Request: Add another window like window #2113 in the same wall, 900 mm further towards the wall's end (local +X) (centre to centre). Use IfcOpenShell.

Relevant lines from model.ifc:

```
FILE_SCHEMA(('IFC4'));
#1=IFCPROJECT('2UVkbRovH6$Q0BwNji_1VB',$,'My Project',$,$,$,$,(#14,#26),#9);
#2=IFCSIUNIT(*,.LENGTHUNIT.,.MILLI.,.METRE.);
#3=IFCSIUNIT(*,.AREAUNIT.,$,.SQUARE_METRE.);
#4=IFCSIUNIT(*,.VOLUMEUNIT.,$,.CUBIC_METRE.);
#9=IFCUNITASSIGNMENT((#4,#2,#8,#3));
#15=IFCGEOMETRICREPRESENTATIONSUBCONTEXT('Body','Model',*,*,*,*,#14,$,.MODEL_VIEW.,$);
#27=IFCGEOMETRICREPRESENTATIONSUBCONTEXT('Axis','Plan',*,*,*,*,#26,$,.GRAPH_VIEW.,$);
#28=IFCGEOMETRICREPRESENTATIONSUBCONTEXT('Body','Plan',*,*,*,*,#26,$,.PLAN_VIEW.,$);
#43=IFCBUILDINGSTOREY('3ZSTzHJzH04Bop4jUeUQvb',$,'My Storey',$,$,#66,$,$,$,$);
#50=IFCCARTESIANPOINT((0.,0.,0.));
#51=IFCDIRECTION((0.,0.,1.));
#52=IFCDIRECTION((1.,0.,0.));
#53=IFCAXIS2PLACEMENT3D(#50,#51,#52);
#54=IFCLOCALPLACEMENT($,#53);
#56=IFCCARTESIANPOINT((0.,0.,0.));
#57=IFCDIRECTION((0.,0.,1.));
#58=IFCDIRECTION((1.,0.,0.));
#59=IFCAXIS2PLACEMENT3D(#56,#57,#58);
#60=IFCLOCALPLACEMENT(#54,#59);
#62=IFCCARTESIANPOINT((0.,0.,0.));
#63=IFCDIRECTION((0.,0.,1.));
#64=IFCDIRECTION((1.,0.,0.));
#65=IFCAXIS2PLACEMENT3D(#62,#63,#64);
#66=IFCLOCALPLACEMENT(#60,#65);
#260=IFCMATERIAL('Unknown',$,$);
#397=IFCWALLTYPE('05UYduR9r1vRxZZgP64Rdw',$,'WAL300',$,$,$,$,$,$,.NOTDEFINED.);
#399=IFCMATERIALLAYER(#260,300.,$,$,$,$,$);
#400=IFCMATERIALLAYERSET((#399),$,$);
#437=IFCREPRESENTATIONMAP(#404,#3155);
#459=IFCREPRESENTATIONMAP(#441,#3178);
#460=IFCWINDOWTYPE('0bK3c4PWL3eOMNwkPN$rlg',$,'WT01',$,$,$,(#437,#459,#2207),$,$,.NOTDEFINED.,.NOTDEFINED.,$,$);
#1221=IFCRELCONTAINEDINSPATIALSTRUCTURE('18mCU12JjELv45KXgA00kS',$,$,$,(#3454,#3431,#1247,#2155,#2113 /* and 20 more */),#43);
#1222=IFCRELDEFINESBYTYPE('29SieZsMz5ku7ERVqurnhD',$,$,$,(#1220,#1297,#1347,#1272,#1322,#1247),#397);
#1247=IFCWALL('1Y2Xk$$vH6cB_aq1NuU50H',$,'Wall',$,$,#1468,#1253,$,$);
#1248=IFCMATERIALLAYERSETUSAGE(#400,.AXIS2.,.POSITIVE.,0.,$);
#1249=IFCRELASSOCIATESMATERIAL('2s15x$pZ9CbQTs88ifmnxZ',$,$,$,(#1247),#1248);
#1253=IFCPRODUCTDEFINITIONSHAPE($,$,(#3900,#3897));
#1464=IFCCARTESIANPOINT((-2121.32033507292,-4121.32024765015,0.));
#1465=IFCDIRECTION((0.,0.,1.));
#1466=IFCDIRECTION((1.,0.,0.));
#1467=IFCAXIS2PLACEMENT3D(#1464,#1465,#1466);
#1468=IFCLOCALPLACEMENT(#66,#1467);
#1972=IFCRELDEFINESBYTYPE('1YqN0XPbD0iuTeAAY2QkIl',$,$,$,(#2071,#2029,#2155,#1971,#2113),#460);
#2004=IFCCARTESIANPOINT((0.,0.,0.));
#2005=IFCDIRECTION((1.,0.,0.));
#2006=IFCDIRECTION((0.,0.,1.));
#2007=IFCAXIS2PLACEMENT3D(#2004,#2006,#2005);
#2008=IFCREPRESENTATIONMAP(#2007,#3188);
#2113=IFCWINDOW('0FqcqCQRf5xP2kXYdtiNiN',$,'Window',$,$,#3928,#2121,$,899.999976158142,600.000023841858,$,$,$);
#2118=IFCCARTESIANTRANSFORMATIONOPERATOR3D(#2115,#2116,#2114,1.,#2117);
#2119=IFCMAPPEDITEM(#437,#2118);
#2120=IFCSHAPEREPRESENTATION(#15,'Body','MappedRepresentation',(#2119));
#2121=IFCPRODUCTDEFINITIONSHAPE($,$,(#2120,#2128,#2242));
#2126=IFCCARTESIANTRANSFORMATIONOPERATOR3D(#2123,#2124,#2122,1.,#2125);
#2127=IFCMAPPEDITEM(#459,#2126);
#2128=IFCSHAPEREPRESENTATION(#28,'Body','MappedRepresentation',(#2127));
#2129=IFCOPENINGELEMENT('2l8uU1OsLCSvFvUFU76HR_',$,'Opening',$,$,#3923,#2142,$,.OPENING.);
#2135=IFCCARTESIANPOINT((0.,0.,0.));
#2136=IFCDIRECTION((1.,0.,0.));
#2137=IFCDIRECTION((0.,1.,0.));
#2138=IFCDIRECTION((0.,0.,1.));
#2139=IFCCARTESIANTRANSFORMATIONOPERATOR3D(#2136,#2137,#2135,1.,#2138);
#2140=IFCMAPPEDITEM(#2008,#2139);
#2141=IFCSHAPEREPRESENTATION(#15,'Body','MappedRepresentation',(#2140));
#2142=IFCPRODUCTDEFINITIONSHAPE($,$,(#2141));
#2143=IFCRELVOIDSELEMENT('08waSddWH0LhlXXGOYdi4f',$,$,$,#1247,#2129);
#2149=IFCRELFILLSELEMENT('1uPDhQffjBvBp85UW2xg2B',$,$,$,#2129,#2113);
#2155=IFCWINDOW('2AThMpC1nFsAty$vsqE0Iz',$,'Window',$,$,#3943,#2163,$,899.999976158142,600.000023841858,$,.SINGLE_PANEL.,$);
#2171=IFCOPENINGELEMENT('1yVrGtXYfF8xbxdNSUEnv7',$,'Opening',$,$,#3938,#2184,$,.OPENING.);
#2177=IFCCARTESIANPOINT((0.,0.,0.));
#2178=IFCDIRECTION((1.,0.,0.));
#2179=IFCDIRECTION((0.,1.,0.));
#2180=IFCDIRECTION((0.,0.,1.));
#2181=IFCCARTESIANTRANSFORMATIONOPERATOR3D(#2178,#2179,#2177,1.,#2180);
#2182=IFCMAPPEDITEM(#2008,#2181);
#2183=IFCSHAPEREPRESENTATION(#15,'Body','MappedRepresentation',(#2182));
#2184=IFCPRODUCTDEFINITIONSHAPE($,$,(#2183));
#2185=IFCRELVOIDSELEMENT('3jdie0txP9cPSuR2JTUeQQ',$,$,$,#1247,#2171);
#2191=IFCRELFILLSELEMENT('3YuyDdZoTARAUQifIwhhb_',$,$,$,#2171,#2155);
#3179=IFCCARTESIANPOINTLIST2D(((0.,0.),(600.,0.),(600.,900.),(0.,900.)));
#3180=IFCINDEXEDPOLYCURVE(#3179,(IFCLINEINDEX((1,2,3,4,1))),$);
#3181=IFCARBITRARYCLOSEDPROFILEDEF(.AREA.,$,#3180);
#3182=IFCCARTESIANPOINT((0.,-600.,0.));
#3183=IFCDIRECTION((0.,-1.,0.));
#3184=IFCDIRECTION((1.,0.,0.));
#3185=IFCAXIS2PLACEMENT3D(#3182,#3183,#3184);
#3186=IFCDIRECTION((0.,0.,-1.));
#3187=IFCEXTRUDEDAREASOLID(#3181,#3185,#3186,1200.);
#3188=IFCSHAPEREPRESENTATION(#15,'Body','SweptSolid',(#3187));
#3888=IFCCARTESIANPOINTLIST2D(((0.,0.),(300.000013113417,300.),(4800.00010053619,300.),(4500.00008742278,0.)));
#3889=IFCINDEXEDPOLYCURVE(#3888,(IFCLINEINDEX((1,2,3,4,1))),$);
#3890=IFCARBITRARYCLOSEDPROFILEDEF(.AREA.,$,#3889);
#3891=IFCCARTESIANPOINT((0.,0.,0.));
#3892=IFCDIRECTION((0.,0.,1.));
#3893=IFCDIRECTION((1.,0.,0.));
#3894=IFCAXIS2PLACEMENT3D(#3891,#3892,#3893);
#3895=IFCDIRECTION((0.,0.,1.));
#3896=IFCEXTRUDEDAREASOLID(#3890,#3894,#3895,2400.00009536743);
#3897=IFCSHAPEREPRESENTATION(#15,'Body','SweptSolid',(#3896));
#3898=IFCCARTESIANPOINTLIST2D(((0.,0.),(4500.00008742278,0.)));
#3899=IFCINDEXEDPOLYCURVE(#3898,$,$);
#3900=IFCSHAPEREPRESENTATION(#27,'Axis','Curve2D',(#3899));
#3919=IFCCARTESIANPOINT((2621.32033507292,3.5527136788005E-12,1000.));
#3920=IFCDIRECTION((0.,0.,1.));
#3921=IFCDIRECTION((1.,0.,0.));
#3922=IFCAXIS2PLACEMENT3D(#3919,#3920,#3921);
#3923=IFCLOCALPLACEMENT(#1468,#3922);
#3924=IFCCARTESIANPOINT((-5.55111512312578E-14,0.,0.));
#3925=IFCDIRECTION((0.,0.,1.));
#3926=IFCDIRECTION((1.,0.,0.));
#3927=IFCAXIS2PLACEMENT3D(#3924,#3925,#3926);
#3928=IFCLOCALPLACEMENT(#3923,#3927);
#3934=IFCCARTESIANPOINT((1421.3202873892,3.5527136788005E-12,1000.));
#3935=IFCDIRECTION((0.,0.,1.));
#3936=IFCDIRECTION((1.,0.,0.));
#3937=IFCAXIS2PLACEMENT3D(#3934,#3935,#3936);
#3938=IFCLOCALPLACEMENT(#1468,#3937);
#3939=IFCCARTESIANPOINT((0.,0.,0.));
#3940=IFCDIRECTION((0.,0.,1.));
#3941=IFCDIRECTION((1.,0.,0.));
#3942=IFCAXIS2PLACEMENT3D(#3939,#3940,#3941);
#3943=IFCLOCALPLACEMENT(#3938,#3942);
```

```python
import ifcopenshell
import ifcopenshell.api.feature
import ifcopenshell.api.geometry
import ifcopenshell.api.root
import ifcopenshell.geom
import ifcopenshell.util.element
import ifcopenshell.util.placement
import ifcopenshell.util.shape

model = ifcopenshell.open("model.ifc")
settings = ifcopenshell.geom.settings()


def volume(element):
    """Net volume in cubic metres, openings subtracted."""
    shape = ifcopenshell.geom.create_shape(settings, element)
    return ifcopenshell.util.shape.get_volume(shape.geometry)


window = model.by_id(2113)
opening = window.FillsVoids[0].RelatingOpeningElement
wall = opening.VoidsElements[0].RelatingBuildingElement
before = volume(wall)
shift = ifcopenshell.util.placement.get_local_placement(wall.ObjectPlacement)[:3, 0] * 900.0

# copy_class copies the void relationship, type, container and properties, but no geometry.
new_opening = ifcopenshell.api.root.copy_class(model, product=opening)
new_opening.Representation = ifcopenshell.util.element.copy_deep(
    model, opening.Representation, exclude=["IfcGeometricRepresentationContext", "IfcRepresentationMap"]
)
new_window = ifcopenshell.api.root.copy_class(model, product=window)
new_window.Representation = ifcopenshell.util.element.copy_deep(
    model, window.Representation, exclude=["IfcGeometricRepresentationContext", "IfcRepresentationMap"]
)
ifcopenshell.api.feature.add_filling(model, opening=new_opening, element=new_window)

for old, new in ((opening, new_opening), (window, new_window)):
    matrix = ifcopenshell.util.placement.get_local_placement(old.ObjectPlacement)
    matrix[:3, 3] += shift
    ifcopenshell.api.geometry.edit_object_placement(model, product=new, matrix=matrix, is_si=False)

after = volume(wall)

print(f"wall volume {before:.3f} -> {after:.3f} m3")

model.write("model_rev.ifc")
```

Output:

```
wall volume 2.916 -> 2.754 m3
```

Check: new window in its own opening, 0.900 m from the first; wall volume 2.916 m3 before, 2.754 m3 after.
